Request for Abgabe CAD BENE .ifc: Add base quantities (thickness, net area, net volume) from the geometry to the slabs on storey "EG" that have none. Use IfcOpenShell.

First a look at what the model holds.

```python
import ifcopenshell
import ifcopenshell.util.element
import ifcopenshell.util.unit

model = ifcopenshell.open("Abgabe CAD BENE .ifc")
print(model.schema)
for unit_type in ("LENGTHUNIT", "AREAUNIT", "VOLUMEUNIT"):
    print(unit_type, ifcopenshell.util.unit.calculate_unit_scale(model, unit_type))
storey = next(s for s in model.by_type("IfcBuildingStorey") if s.Name == "EG")
slabs = [e for e in ifcopenshell.util.element.get_decomposition(storey) if e.is_a("IfcSlab")]
for e in sorted(slabs, key=lambda e: e.id()):
    print(e.id(), e.is_a(), e.Name, list(ifcopenshell.util.element.get_psets(e, qtos_only=True)), sep=" | ")
```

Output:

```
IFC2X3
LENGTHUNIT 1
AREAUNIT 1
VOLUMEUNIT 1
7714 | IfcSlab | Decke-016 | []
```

```python
import ifcopenshell
import ifcopenshell.api.pset
import ifcopenshell.geom
import ifcopenshell.util.element
import ifcopenshell.util.shape
import ifcopenshell.util.unit

model = ifcopenshell.open("Abgabe CAD BENE .ifc")
unit_scale = ifcopenshell.util.unit.calculate_unit_scale(model)
area_scale = ifcopenshell.util.unit.calculate_unit_scale(model, "AREAUNIT")
volume_scale = ifcopenshell.util.unit.calculate_unit_scale(model, "VOLUMEUNIT")
settings = ifcopenshell.geom.settings()

storey = next(s for s in model.by_type("IfcBuildingStorey") if s.Name == "EG")
slabs = [e for e in ifcopenshell.util.element.get_decomposition(storey) if e.is_a("IfcSlab")]

for e in sorted(slabs, key=lambda e: e.id()):
    if ifcopenshell.util.element.get_psets(e, qtos_only=True, should_inherit=False):
        continue
    # Geometry comes back in metres, in the element's own axes.
    shape = ifcopenshell.geom.create_shape(settings, e)
    values = {
        "Width": ifcopenshell.util.shape.get_z(shape.geometry) / unit_scale,
        "NetArea": ifcopenshell.util.shape.get_footprint_area(shape.geometry) / area_scale,
        "NetVolume": ifcopenshell.util.shape.get_volume(shape.geometry) / volume_scale,
    }
    qto = ifcopenshell.api.pset.add_qto(model, product=e, name="BaseQuantities")
    ifcopenshell.api.pset.edit_qto(model, qto=qto, properties=values)
    print(e.id(), {k: round(v, 3) for k, v in values.items()})

model.write("Abgabe CAD BENE -out.ifc")
```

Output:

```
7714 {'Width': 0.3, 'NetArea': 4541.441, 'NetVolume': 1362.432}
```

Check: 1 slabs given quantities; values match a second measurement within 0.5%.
